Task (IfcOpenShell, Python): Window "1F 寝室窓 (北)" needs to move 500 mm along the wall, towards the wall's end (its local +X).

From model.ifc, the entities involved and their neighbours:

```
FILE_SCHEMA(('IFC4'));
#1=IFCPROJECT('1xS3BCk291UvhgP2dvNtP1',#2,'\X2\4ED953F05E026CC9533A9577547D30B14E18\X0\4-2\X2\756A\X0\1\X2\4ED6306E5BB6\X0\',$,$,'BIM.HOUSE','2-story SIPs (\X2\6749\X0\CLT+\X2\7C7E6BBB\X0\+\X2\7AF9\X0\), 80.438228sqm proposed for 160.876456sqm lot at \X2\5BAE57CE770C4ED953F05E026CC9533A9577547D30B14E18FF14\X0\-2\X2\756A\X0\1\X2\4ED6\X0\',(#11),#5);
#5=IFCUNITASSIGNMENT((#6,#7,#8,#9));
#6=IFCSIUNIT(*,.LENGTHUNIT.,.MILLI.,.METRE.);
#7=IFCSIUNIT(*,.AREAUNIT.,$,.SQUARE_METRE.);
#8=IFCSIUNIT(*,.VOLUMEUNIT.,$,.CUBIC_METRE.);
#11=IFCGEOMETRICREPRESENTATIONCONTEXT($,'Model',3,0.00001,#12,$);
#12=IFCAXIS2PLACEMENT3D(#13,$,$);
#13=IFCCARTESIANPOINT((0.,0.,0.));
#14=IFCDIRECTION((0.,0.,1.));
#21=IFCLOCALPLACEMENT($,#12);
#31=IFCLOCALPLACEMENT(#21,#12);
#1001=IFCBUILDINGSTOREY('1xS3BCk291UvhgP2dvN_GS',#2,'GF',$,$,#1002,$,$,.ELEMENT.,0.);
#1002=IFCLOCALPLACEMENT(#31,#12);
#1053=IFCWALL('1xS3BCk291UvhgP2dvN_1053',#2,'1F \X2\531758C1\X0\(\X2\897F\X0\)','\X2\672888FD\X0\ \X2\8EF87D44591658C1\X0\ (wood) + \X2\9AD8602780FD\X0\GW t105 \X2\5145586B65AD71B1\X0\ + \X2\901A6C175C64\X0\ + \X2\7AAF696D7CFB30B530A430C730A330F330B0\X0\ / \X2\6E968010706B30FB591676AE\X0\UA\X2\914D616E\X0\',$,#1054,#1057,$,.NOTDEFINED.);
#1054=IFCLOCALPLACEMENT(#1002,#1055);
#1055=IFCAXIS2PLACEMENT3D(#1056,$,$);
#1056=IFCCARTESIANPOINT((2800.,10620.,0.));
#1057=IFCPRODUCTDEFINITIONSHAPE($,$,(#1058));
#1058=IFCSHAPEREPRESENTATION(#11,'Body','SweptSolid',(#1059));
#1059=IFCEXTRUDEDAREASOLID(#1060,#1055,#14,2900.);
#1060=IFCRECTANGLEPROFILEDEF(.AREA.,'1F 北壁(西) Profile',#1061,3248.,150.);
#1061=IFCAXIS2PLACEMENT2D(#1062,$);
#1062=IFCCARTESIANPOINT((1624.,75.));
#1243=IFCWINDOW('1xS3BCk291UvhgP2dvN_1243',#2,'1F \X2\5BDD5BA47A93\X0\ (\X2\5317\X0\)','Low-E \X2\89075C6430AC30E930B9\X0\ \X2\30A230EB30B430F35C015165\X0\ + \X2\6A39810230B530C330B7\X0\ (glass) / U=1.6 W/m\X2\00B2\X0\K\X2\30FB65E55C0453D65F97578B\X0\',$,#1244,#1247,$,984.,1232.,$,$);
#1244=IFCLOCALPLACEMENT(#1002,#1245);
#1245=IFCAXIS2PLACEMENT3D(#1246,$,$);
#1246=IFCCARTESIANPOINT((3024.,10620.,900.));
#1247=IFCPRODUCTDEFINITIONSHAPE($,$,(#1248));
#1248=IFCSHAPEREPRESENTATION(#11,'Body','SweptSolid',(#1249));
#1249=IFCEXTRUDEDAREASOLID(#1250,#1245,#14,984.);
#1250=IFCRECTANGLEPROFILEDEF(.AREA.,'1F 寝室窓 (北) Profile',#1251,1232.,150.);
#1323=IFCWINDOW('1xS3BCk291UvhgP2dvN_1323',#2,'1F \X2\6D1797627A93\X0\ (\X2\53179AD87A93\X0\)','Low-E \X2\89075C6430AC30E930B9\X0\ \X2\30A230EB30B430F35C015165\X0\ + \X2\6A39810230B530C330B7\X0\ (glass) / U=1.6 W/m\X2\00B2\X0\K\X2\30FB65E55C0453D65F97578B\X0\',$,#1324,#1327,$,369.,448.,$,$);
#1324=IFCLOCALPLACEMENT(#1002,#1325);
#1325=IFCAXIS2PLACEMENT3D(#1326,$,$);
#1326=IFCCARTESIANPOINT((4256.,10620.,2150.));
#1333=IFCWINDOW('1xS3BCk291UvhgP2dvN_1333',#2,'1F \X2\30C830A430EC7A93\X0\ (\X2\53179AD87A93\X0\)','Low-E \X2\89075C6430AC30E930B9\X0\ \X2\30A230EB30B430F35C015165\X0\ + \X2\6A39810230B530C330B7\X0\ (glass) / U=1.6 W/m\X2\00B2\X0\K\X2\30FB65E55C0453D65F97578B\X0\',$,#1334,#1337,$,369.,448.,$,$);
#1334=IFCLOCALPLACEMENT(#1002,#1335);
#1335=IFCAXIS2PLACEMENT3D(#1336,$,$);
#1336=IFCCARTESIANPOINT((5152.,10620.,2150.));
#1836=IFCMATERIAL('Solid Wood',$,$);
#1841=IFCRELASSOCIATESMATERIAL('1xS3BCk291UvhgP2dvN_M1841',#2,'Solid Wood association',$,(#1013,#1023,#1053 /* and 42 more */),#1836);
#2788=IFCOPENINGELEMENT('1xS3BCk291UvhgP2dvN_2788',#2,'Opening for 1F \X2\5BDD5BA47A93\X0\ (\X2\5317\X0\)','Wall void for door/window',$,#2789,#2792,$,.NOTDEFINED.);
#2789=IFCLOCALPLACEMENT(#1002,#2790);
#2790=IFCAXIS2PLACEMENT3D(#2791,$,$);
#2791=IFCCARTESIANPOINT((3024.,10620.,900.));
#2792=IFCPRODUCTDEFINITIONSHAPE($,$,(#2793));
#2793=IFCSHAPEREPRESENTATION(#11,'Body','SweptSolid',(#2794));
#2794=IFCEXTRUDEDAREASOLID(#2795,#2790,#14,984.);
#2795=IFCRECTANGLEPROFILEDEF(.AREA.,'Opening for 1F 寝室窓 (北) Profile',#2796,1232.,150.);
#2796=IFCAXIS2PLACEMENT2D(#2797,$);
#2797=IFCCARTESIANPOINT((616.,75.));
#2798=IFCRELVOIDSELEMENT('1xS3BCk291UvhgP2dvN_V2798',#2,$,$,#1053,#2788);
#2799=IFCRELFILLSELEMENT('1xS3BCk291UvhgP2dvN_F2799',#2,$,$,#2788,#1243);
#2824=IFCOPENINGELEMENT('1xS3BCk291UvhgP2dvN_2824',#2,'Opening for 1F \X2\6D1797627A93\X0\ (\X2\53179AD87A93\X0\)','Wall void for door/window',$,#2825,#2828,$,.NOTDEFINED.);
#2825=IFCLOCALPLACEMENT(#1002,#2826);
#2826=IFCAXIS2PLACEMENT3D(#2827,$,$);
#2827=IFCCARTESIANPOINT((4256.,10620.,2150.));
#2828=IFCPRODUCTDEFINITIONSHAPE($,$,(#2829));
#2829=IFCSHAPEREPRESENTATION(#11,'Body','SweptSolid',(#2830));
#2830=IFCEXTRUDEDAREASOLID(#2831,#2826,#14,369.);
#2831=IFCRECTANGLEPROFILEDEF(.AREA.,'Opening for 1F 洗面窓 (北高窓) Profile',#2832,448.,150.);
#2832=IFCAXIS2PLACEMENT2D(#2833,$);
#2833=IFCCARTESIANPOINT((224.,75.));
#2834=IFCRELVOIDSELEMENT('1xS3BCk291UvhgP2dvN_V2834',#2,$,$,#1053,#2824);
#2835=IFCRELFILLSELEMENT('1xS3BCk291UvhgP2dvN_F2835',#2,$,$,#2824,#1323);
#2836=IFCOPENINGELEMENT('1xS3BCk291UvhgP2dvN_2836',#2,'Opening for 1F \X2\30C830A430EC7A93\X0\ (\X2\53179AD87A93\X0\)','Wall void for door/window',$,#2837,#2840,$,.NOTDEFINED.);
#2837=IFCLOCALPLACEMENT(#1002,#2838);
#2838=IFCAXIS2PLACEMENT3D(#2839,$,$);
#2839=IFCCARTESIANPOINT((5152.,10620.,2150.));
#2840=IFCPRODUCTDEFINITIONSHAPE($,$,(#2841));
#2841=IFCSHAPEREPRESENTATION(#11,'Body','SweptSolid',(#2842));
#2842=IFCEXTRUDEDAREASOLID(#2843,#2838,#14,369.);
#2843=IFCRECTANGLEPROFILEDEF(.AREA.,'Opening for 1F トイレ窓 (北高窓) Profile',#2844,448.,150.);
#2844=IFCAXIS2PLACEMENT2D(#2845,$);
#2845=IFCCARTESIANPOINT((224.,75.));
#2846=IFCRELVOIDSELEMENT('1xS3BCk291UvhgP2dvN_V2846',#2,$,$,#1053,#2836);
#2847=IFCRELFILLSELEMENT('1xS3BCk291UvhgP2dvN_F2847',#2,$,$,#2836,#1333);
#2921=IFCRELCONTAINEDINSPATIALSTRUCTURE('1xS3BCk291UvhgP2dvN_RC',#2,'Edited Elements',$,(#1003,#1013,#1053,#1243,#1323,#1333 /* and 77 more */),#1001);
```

```python
import ifcopenshell
import ifcopenshell.api.geometry
import ifcopenshell.util.placement
import ifcopenshell.util.unit

model = ifcopenshell.open("model.ifc")
unit_scale = ifcopenshell.util.unit.calculate_unit_scale(model)

window = model.by_guid("1xS3BCk291UvhgP2dvN_1243")
opening = window.FillsVoids[0].RelatingOpeningElement
wall = opening.VoidsElements[0].RelatingBuildingElement

wall_matrix = ifcopenshell.util.placement.get_local_placement(wall.ObjectPlacement)
shift = wall_matrix[:3, 0] * 0.5 / unit_scale
before = ifcopenshell.util.placement.get_local_placement(window.ObjectPlacement)[:3, 3].copy()

# The window is not placed relative to its opening, so move both.
for product in (opening, window):
    matrix = ifcopenshell.util.placement.get_local_placement(product.ObjectPlacement)
    matrix[:3, 3] += shift
    ifcopenshell.api.geometry.edit_object_placement(model, product=product, matrix=matrix, is_si=False)

after = ifcopenshell.util.placement.get_local_placement(window.ObjectPlacement)[:3, 3]
print("window moved by", (after - before).round(3) + 0.0)

model.write("model-out.ifc")
```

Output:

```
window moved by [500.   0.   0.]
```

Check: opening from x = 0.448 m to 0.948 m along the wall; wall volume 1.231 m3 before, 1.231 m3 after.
